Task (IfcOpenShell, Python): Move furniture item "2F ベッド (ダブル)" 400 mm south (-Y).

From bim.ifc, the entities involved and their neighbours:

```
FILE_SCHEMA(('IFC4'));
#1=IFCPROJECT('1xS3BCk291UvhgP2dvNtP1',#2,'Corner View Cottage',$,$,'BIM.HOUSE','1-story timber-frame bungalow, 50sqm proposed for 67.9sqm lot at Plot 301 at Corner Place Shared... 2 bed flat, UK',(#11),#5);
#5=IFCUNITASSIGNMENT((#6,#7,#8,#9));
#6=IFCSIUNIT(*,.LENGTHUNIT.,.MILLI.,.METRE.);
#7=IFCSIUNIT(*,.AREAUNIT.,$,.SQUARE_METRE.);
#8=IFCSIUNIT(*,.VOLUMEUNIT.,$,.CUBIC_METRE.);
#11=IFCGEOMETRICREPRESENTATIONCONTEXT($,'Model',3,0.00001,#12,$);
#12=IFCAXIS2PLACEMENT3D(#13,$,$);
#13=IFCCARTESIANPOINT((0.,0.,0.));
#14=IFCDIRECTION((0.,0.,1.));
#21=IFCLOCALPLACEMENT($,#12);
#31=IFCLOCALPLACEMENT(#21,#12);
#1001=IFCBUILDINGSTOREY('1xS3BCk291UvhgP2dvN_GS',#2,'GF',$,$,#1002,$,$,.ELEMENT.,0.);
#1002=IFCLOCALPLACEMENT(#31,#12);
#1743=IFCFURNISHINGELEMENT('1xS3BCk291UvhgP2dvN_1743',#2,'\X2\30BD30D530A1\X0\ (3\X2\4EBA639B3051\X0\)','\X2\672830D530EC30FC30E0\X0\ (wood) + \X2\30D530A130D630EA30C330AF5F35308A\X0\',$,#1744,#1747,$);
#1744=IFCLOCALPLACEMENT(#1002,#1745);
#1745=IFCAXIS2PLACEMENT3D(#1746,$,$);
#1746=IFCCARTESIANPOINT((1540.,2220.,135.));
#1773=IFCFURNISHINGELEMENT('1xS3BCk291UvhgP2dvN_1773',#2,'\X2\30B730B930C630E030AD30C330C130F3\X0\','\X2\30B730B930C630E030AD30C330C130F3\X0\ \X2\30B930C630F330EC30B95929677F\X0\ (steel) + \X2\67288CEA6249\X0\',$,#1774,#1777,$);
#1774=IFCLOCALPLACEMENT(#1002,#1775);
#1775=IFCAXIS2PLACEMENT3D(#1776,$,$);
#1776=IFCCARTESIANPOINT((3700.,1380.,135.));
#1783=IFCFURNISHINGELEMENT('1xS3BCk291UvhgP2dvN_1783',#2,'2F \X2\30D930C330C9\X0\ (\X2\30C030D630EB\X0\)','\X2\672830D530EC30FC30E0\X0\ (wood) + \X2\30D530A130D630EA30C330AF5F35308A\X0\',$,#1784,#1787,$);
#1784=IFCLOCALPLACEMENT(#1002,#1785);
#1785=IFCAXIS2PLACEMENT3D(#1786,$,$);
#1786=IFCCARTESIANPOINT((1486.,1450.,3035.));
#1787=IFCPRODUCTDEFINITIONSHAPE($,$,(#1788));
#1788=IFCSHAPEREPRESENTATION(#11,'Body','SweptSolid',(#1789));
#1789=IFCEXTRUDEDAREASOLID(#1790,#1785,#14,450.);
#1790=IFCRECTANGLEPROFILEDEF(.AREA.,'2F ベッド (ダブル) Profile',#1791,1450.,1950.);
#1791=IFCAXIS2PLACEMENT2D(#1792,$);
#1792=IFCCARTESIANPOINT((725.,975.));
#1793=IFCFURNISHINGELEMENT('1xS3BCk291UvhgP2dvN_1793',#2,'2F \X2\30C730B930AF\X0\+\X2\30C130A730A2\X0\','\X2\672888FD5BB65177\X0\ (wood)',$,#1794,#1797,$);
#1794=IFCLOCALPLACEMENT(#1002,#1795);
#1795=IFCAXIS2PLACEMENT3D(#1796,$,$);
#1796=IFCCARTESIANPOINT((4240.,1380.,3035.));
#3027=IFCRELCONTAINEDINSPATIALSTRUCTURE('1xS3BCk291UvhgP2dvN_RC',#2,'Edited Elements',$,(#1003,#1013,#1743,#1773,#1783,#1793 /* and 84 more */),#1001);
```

```python
import ifcopenshell
import ifcopenshell.api.geometry
import ifcopenshell.util.placement
import ifcopenshell.util.unit

model = ifcopenshell.open("bim.ifc")
unit_scale = ifcopenshell.util.unit.calculate_unit_scale(model)

item = model.by_guid("1xS3BCk291UvhgP2dvN_1783")
matrix = ifcopenshell.util.placement.get_local_placement(item.ObjectPlacement)
matrix[1, 3] -= 0.4 / unit_scale
ifcopenshell.api.geometry.edit_object_placement(model, product=item, matrix=matrix, is_si=False)

print(ifcopenshell.util.placement.get_local_placement(item.ObjectPlacement).round(3) + 0.0)

model.write("bim_rev.ifc")
```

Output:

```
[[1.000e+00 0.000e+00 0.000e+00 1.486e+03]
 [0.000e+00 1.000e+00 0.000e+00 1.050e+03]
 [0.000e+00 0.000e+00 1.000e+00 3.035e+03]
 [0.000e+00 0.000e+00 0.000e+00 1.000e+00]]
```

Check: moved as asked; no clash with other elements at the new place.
